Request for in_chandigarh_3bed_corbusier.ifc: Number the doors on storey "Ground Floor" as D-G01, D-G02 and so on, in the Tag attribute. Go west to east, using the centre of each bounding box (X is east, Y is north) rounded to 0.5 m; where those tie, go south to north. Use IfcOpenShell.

First a look at what the model holds.

```python
import ifcopenshell
import ifcopenshell.util.element
import ifcopenshell.util.placement

model = ifcopenshell.open("in_chandigarh_3bed_corbusier.ifc")
print(model.schema)
storey = next(s for s in model.by_type("IfcBuildingStorey") if s.Name == "Ground Floor")
doors = [e for e in ifcopenshell.util.element.get_decomposition(storey) if e.is_a("IfcDoor")]
for e in sorted(doors, key=lambda e: e.id()):
    origin = ifcopenshell.util.placement.get_local_placement(e.ObjectPlacement)[:3, 3]
    print(e.id(), e.Tag, e.Name, origin.round(2) + 0.0, sep=" | ")
```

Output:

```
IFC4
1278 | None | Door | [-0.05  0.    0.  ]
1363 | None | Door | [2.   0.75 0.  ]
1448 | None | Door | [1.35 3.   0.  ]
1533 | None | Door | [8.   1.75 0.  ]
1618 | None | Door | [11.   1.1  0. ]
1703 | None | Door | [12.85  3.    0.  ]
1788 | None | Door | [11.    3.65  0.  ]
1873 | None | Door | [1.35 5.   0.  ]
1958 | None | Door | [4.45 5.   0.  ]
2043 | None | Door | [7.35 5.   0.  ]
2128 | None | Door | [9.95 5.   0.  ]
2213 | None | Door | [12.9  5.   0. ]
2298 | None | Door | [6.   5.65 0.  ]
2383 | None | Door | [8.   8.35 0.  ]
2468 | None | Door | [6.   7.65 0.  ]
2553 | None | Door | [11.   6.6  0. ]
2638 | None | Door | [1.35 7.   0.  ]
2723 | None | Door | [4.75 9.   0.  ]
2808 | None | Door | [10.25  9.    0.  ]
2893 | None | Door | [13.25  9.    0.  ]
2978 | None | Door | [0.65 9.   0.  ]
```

```python
import ifcopenshell
import ifcopenshell.geom
import ifcopenshell.util.element
import ifcopenshell.util.shape

model = ifcopenshell.open("in_chandigarh_3bed_corbusier.ifc")
settings = ifcopenshell.geom.settings()
settings.set("use-world-coords", True)


def centre(element):
    shape = ifcopenshell.geom.create_shape(settings, element)
    return ifcopenshell.util.shape.get_bbox_centroid(shape.geometry)


storey = next(s for s in model.by_type("IfcBuildingStorey") if s.Name == "Ground Floor")
doors = [e for e in ifcopenshell.util.element.get_decomposition(storey) if e.is_a("IfcDoor")]

# Insertion points can sit at a corner or the storey origin, so sort by the geometry (in metres).
centres = {e: centre(e) for e in doors}
doors.sort(key=lambda e: (round(centres[e][0] / 0.5), centres[e][1]))

for i, e in enumerate(doors, start=1):
    number = f"D-G{i:02d}"
    e.Tag = number
    print(e.id(), number)

model.write("in_chandigarh_3bed_corbusier_rev.ifc")
```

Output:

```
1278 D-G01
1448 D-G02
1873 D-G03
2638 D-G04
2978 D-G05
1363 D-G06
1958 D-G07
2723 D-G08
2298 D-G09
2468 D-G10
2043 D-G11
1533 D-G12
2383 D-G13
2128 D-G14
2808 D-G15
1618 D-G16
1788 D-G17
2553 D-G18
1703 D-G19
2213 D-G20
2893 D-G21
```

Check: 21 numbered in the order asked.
